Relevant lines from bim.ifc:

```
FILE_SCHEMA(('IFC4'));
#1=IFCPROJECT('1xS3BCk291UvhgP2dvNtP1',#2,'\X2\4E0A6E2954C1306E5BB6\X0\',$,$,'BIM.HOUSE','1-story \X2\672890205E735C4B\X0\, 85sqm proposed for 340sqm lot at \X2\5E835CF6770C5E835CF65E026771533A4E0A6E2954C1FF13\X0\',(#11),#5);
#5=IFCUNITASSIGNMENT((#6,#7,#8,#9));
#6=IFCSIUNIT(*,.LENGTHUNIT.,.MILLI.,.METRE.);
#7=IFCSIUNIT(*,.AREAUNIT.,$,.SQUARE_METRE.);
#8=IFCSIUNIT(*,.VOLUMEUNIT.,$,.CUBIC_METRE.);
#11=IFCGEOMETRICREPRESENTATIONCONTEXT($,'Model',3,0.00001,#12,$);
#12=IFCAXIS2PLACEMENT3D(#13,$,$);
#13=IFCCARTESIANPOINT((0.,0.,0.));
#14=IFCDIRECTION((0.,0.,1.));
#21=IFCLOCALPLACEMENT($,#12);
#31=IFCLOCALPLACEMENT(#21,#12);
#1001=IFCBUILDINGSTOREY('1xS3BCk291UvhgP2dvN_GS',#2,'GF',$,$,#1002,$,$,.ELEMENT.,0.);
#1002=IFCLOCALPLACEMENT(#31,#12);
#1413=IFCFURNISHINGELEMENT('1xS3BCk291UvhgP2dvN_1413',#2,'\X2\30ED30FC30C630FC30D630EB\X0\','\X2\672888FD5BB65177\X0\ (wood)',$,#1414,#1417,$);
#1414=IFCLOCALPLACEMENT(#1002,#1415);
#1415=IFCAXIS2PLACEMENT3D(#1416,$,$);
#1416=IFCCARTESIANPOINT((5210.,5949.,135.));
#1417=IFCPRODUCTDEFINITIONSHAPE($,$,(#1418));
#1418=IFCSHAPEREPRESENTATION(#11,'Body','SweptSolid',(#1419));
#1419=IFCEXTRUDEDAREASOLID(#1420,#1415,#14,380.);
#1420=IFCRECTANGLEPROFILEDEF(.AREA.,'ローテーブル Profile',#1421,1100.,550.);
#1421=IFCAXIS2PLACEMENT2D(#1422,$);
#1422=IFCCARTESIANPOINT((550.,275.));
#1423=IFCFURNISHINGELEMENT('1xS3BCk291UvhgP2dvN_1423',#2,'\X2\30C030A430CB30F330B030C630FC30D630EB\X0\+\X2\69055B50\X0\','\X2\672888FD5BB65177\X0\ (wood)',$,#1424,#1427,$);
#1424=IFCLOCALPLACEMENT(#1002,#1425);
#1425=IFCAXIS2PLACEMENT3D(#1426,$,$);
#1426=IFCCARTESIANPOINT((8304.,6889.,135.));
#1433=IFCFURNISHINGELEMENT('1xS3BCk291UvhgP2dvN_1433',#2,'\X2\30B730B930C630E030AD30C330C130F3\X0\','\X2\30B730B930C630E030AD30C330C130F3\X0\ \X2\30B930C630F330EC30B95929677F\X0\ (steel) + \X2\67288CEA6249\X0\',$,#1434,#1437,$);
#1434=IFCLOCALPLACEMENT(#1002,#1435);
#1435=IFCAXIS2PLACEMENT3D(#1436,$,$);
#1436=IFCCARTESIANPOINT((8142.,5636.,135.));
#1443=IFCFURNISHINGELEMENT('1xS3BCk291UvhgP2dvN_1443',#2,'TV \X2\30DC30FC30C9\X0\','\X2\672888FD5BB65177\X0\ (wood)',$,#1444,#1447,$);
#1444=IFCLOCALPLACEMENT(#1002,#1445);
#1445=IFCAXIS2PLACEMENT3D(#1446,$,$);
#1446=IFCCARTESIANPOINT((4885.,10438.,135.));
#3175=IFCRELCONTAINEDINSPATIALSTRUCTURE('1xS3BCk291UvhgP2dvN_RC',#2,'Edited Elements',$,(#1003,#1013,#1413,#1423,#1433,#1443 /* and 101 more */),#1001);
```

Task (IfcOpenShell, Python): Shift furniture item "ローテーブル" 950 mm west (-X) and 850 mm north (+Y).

```python
import ifcopenshell
import ifcopenshell.api.geometry
import ifcopenshell.util.placement
import ifcopenshell.util.unit

model = ifcopenshell.open("bim.ifc")
unit_scale = ifcopenshell.util.unit.calculate_unit_scale(model)

item = model.by_guid("1xS3BCk291UvhgP2dvN_1413")
matrix = ifcopenshell.util.placement.get_local_placement(item.ObjectPlacement)
matrix[0, 3] -= 0.95 / unit_scale
matrix[1, 3] += 0.85 / unit_scale
ifcopenshell.api.geometry.edit_object_placement(model, product=item, matrix=matrix, is_si=False)

print(ifcopenshell.util.placement.get_local_placement(item.ObjectPlacement).round(3) + 0.0)

model.write("bim_updated.ifc")
```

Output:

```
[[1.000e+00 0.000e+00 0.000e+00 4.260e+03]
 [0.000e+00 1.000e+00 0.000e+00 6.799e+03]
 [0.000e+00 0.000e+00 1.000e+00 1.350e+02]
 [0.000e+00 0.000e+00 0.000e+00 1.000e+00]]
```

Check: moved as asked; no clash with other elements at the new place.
